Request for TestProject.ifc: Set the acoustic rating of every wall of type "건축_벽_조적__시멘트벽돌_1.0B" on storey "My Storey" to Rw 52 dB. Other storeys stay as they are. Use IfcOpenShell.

First a look at what the model holds.

```python
import ifcopenshell
import ifcopenshell.util.element

model = ifcopenshell.open("TestProject.ifc")
print(model.schema)
storey = next(s for s in model.by_type("IfcBuildingStorey") if s.Name == "My Storey")
walls = [e for e in ifcopenshell.util.element.get_decomposition(storey) if e.is_a("IfcWall")]
seen = {}
for e in walls:
    element_type = ifcopenshell.util.element.get_type(e)
    key = (element_type.Name if element_type != e and element_type else None, ifcopenshell.util.element.get_pset(e, "Pset_WallCommon", "AcousticRating"))
    seen[key] = seen.get(key, 0) + 1
for (name, value), count in sorted(seen.items(), key=str):
    print(count, "x", name, "|", value)
```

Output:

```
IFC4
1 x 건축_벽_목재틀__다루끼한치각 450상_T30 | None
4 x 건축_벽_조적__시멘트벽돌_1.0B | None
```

```python
import ifcopenshell
import ifcopenshell.api.pset
import ifcopenshell.util.element

model = ifcopenshell.open("TestProject.ifc")

storey = next(s for s in model.by_type("IfcBuildingStorey") if s.Name == "My Storey")
walls = [e for e in ifcopenshell.util.element.get_decomposition(storey) if e.is_a("IfcWall")]

count = 0
for e in walls:
    element_type = ifcopenshell.util.element.get_type(e)
    if element_type in (None, e) or element_type.Name != "건축_벽_조적__시멘트벽돌_1.0B":
        continue
    # add_pset returns the element's existing set when there is one.
    pset = ifcopenshell.api.pset.add_pset(model, product=e, name="Pset_WallCommon")
    ifcopenshell.api.pset.edit_pset(model, pset=pset, properties={"AcousticRating": "Rw 52 dB"})
    count += 1

print(count, "walls updated")

model.write("TestProject_v2.ifc")
```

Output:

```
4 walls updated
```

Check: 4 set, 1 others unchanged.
